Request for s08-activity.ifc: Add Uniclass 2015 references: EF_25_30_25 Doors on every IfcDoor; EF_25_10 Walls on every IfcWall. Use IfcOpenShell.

First a look at what the model holds.

```python
import ifcopenshell

model = ifcopenshell.open("s08-activity.ifc")
print(model.schema)
print("classifications:", [c.Name for c in model.by_type("IfcClassification")])
for ifc_class in ("IfcDoor", "IfcRoof", "IfcStair", "IfcWall", "IfcWindow"):
    print(ifc_class, len(model.by_type(ifc_class)))
```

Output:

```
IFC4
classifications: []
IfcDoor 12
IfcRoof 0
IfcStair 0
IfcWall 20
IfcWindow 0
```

```python
import ifcopenshell
import ifcopenshell.api.classification

model = ifcopenshell.open("s08-activity.ifc")

system = ifcopenshell.api.classification.add_classification(model, classification="Uniclass 2015")

codes = {
    "IfcDoor": ("EF_25_30_25", "Doors"),
    "IfcWall": ("EF_25_10", "Walls"),
}
for ifc_class, (code, name) in codes.items():
    products = model.by_type(ifc_class)
    ifcopenshell.api.classification.add_reference(
        model, products=products, classification=system, identification=code, name=name
    )
    print(code, len(products))

model.write("s08-activity_rev.ifc")
```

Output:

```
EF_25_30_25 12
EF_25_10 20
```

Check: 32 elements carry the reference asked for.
